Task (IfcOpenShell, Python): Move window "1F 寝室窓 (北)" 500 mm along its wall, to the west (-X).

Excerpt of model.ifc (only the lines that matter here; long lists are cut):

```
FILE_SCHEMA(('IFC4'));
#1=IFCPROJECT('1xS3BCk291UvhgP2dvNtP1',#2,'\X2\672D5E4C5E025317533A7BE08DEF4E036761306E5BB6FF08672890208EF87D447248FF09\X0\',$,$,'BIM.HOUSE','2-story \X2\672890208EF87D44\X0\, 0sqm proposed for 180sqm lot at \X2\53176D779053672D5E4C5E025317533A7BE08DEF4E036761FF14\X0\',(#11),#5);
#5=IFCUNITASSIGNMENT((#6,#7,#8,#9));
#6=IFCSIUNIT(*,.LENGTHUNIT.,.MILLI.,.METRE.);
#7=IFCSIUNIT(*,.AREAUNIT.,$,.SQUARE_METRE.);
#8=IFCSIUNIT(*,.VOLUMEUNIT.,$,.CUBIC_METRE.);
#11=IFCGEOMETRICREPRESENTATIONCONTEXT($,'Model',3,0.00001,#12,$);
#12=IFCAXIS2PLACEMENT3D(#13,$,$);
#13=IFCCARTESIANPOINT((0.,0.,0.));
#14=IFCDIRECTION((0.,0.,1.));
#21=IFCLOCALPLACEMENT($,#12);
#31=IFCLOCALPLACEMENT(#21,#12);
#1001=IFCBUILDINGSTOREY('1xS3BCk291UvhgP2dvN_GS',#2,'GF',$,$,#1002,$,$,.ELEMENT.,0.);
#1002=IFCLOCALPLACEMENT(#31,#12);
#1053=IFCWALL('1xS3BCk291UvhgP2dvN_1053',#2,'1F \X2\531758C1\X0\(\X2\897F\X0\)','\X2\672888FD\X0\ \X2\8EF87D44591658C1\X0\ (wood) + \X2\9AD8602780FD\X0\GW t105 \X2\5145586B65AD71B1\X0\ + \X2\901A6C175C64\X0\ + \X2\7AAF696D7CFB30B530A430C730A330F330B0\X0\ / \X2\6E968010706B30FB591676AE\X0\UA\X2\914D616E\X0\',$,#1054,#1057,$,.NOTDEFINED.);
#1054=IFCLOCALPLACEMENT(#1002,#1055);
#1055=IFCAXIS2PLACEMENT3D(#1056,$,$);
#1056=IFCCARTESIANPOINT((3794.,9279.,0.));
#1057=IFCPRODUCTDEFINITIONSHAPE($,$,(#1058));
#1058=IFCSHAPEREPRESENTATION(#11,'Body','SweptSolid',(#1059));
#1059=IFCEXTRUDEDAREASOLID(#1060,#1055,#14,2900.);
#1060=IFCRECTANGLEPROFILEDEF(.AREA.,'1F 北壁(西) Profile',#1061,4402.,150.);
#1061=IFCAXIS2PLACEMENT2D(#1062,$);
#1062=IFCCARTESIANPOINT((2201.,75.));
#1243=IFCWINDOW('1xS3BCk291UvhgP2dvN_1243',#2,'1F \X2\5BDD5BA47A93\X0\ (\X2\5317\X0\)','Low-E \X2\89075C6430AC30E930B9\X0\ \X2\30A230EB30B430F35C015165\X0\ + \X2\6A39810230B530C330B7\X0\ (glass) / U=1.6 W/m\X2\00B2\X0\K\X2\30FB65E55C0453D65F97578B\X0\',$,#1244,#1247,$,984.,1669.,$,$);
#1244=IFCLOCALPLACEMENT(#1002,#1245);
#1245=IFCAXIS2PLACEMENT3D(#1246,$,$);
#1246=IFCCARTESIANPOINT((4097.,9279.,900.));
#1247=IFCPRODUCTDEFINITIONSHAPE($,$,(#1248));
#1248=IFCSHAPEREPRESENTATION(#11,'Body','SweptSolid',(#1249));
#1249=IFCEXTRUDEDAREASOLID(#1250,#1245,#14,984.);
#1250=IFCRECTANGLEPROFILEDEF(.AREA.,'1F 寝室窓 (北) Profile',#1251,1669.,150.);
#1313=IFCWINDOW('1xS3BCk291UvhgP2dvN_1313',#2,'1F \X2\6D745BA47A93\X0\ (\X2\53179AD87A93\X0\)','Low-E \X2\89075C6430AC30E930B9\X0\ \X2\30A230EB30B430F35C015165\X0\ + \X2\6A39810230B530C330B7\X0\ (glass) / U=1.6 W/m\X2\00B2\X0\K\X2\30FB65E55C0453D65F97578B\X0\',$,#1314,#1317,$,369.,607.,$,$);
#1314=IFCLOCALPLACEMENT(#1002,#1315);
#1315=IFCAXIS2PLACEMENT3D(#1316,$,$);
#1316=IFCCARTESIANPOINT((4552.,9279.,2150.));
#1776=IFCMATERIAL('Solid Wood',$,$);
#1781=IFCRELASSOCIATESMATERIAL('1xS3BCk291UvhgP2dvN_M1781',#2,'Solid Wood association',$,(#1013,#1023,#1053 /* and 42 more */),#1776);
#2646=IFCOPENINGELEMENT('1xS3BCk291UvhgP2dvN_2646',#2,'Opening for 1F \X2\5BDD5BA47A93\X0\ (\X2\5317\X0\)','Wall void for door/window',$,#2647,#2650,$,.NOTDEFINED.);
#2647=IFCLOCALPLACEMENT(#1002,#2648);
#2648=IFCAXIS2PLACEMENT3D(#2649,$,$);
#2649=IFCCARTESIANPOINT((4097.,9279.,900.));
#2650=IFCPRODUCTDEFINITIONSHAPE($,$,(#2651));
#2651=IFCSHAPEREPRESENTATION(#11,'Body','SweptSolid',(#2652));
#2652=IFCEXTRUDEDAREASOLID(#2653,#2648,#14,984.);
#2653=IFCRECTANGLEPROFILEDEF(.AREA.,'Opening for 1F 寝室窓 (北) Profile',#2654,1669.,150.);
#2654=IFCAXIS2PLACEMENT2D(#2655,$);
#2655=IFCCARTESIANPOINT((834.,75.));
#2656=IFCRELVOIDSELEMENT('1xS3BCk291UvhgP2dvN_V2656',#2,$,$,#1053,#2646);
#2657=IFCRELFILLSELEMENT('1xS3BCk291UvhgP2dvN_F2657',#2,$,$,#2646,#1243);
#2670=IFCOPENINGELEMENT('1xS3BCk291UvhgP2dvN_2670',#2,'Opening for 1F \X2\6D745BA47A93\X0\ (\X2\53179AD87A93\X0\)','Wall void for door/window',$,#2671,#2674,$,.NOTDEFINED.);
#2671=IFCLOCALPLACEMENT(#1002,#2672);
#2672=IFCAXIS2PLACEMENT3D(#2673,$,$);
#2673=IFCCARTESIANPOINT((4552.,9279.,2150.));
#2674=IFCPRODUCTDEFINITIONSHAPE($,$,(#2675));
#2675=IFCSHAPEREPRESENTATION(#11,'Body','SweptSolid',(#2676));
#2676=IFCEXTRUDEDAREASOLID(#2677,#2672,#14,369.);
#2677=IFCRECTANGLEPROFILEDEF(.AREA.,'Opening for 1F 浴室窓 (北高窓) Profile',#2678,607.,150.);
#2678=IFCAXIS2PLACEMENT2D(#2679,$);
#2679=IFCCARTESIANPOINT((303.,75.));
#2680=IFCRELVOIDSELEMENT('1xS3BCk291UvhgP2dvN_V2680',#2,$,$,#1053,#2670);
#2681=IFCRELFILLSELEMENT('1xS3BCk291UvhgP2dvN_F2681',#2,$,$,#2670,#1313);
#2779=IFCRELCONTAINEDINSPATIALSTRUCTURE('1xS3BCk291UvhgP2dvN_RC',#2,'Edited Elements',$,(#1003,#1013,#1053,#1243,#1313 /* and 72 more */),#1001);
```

```python
import ifcopenshell
import ifcopenshell.api.geometry
import ifcopenshell.util.placement
import ifcopenshell.util.unit

model = ifcopenshell.open("model.ifc")
unit_scale = ifcopenshell.util.unit.calculate_unit_scale(model)

window = model.by_guid("1xS3BCk291UvhgP2dvN_1243")
opening = window.FillsVoids[0].RelatingOpeningElement
wall = opening.VoidsElements[0].RelatingBuildingElement

wall_matrix = ifcopenshell.util.placement.get_local_placement(wall.ObjectPlacement)
shift = wall_matrix[:3, 0] * -0.5 / unit_scale
before = ifcopenshell.util.placement.get_local_placement(window.ObjectPlacement)[:3, 3].copy()

# The window is not placed relative to its opening, so move both.
for product in (opening, window):
    matrix = ifcopenshell.util.placement.get_local_placement(product.ObjectPlacement)
    matrix[:3, 3] += shift
    ifcopenshell.api.geometry.edit_object_placement(model, product=product, matrix=matrix, is_si=False)

after = ifcopenshell.util.placement.get_local_placement(window.ObjectPlacement)[:3, 3]
print("window moved by", (after - before).round(3) + 0.0)

model.write("model-out.ifc")
```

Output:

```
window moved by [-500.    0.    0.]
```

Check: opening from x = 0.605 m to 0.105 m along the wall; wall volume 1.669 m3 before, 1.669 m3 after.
